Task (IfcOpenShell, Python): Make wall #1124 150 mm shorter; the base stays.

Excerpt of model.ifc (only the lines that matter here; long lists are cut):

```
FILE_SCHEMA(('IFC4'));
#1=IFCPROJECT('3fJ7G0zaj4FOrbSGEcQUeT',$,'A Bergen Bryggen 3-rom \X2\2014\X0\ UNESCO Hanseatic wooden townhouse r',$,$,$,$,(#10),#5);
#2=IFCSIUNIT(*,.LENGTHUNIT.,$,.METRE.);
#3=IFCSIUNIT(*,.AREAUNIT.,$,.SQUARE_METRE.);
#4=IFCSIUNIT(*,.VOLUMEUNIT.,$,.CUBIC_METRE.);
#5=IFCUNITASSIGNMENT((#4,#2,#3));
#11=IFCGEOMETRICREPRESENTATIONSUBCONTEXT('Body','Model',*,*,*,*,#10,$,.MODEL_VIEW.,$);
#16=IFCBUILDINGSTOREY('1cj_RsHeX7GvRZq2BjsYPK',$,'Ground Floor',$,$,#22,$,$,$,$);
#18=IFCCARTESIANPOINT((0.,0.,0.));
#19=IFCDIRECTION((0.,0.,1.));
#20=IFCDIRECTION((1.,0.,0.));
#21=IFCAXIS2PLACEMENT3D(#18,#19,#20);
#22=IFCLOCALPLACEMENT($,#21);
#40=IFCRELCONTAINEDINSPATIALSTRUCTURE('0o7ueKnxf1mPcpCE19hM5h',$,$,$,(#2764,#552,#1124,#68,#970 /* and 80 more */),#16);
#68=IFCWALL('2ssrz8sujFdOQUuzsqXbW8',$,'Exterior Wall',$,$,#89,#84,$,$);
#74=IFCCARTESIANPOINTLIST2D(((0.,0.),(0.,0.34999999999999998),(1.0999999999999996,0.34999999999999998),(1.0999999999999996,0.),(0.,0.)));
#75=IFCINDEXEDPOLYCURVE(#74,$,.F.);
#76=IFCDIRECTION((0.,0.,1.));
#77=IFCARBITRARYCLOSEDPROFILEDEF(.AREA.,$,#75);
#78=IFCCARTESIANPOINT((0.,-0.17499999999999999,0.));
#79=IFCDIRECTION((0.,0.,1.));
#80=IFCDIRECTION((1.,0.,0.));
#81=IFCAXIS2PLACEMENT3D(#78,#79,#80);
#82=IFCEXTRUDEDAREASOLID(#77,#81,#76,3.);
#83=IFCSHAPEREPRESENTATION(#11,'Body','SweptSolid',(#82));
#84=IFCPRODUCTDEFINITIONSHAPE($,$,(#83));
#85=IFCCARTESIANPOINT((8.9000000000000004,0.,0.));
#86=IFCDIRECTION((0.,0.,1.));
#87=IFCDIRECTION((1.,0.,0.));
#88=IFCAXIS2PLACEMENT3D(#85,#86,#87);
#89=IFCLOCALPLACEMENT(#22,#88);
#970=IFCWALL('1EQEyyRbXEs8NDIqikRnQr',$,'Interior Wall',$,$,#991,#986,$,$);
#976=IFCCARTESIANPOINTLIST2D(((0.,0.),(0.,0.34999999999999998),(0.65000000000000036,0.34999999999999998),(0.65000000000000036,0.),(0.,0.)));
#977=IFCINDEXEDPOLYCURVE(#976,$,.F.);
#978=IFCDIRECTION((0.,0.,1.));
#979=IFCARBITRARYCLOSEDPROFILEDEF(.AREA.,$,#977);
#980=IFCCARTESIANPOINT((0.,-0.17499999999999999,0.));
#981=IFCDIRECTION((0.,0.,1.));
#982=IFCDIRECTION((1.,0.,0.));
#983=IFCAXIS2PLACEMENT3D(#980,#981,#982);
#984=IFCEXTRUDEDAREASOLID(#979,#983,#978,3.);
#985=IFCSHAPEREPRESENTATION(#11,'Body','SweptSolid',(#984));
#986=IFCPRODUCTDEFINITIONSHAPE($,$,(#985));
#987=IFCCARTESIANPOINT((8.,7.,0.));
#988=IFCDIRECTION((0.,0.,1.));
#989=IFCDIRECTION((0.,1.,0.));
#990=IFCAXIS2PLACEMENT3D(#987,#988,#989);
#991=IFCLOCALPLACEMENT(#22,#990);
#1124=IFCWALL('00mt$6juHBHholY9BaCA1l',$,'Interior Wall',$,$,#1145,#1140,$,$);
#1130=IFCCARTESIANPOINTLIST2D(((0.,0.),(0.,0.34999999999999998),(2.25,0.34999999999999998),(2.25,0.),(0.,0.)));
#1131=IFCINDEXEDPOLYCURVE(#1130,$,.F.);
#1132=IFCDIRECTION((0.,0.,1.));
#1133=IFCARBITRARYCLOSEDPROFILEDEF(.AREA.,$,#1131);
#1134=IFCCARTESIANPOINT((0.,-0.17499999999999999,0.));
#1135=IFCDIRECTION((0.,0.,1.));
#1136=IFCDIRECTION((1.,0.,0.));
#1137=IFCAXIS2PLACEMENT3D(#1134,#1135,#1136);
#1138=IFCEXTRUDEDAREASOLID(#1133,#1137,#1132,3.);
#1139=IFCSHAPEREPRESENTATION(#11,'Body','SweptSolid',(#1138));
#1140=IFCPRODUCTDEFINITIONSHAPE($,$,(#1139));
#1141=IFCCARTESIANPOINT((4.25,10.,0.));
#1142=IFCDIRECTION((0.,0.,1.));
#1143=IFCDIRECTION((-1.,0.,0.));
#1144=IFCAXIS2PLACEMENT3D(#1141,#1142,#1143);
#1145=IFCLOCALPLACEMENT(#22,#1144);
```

```python
import ifcopenshell
import ifcopenshell.geom
import ifcopenshell.util.representation
import ifcopenshell.util.shape
import ifcopenshell.util.unit

model = ifcopenshell.open("model.ifc")
unit_scale = ifcopenshell.util.unit.calculate_unit_scale(model)
settings = ifcopenshell.geom.settings()


def volume(element):
    """Net volume in cubic metres, openings subtracted."""
    shape = ifcopenshell.geom.create_shape(settings, element)
    return ifcopenshell.util.shape.get_volume(shape.geometry)


wall = model.by_id(1124)
before = volume(wall)

body = ifcopenshell.util.representation.get_representation(wall, "Model", "Body")
solid = body.Items[0]
old_height = solid.Depth
solid.Depth -= 0.15 / unit_scale
after = volume(wall)

print(f"height {old_height:g} -> {solid.Depth:g}, volume {before:.3f} -> {after:.3f} m3")

model.write("model_rev.ifc")
```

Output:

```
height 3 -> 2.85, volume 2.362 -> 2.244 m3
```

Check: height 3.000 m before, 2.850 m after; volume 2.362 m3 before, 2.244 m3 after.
